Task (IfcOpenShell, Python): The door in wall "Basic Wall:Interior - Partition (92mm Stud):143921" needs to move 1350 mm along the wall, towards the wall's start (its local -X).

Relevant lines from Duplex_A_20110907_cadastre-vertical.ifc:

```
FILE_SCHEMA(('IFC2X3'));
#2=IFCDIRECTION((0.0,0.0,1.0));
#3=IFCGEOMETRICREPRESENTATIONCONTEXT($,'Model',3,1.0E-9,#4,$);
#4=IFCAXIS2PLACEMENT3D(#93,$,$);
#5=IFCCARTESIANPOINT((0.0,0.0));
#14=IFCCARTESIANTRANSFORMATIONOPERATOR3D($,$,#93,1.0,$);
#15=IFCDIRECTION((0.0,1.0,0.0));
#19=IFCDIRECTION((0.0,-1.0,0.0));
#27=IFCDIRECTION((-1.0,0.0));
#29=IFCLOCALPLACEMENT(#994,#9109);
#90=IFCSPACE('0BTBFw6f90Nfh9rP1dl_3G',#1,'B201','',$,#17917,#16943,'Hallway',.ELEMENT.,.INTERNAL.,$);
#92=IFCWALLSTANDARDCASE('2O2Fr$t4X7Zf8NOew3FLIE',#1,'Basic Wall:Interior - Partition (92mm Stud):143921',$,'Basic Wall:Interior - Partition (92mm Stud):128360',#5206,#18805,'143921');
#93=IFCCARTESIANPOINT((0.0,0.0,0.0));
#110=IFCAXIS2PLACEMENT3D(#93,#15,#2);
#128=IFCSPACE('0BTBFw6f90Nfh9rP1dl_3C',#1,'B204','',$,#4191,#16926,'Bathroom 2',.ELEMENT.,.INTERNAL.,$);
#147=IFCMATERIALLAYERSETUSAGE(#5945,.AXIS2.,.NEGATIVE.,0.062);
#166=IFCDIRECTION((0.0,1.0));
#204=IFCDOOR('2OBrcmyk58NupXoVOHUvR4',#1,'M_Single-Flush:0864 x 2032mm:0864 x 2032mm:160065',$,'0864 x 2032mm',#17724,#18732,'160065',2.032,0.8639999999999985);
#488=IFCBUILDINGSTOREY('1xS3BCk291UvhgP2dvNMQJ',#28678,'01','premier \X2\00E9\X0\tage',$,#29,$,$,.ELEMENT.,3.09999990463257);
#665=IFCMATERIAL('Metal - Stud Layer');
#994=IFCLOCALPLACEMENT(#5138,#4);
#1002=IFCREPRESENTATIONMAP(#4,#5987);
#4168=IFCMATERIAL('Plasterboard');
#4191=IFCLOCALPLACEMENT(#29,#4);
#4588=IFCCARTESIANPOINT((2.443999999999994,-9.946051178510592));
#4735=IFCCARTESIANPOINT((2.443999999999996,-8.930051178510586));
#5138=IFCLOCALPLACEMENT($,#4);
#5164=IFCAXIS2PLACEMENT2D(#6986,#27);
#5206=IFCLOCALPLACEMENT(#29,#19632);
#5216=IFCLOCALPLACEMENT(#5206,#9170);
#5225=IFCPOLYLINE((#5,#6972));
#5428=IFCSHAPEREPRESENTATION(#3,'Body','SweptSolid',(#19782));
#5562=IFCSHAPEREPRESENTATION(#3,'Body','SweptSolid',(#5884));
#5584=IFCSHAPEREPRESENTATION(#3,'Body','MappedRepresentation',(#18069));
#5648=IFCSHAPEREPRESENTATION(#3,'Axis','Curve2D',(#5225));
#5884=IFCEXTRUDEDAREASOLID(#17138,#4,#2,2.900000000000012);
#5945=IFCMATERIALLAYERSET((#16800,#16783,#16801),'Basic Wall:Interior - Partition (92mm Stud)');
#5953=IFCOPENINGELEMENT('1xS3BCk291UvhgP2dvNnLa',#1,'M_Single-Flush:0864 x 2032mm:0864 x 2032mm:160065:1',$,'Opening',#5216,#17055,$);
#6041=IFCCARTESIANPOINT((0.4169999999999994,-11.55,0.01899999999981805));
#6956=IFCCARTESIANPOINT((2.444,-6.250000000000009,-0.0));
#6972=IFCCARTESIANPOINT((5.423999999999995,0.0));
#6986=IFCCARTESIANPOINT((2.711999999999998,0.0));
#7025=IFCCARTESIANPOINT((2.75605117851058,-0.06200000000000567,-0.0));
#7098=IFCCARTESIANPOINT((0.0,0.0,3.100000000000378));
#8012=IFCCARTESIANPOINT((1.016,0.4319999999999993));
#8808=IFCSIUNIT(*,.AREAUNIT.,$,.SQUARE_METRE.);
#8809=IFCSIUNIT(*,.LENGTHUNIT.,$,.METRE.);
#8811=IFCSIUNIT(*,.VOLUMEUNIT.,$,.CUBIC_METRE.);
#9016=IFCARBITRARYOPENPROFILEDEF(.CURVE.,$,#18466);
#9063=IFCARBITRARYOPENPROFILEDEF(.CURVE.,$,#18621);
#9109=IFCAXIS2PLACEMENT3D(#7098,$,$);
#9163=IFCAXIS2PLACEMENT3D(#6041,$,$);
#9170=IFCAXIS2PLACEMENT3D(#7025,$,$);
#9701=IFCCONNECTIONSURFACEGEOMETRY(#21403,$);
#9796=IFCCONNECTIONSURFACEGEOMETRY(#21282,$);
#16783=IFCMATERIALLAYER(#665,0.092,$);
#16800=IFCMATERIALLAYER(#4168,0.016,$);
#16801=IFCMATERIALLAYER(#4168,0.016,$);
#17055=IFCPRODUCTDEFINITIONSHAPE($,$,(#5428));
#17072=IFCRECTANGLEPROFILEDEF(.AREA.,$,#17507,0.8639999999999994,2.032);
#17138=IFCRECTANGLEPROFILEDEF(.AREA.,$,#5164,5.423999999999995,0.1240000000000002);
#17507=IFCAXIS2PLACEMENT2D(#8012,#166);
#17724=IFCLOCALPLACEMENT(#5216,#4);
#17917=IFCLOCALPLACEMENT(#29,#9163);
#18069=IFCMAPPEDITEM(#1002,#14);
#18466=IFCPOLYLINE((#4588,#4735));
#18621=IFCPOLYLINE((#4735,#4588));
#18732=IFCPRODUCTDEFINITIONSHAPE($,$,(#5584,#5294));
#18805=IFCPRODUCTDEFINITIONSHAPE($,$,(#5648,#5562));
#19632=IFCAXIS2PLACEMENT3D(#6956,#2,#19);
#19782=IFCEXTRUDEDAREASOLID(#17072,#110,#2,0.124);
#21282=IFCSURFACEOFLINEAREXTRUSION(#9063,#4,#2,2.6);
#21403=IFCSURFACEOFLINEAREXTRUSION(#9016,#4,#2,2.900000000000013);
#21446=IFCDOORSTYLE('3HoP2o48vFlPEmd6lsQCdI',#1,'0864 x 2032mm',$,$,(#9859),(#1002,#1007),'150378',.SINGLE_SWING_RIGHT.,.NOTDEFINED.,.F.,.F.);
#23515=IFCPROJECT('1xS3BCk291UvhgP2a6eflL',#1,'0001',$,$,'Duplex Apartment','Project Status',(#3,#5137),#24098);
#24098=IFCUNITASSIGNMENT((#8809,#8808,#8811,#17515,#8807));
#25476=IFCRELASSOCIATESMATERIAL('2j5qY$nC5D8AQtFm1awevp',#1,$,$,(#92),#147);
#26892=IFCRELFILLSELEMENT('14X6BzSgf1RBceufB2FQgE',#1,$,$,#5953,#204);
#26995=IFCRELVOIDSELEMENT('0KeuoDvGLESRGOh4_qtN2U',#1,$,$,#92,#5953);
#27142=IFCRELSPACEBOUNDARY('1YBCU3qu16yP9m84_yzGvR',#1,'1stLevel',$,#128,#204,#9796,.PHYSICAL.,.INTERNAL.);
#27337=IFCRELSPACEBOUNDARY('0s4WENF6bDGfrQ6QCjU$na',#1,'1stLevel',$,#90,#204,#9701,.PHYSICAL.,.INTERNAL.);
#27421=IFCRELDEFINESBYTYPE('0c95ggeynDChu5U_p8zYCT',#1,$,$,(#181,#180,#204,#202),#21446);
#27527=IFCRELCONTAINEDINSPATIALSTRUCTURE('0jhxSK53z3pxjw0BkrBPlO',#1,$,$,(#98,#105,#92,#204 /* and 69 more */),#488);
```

```python
import numpy as np
import ifcopenshell
import ifcopenshell.api.geometry
import ifcopenshell.util.placement

model = ifcopenshell.open("Duplex_A_20110907_cadastre-vertical.ifc")

door = model.by_guid("2OBrcmyk58NupXoVOHUvR4")
opening = door.FillsVoids[0].RelatingOpeningElement
wall = opening.VoidsElements[0].RelatingBuildingElement

wall_matrix = ifcopenshell.util.placement.get_local_placement(wall.ObjectPlacement)
shift = wall_matrix[:3, 0] * -1.35
before = ifcopenshell.util.placement.get_local_placement(door.ObjectPlacement)[:3, 3].copy()

# The door is placed relative to its opening, so it follows when the opening moves.
matrix = ifcopenshell.util.placement.get_local_placement(opening.ObjectPlacement)
matrix[:3, 3] += shift
ifcopenshell.api.geometry.edit_object_placement(
    model, product=opening, matrix=matrix, is_si=False, should_transform_children=True
)

# Space boundary surfaces are stored in each space's coordinates; move them too.
for rel in door.ProvidesBoundaries:
    if not rel.ConnectionGeometry:
        continue
    surface = rel.ConnectionGeometry.SurfaceOnRelatingElement
    space_matrix = ifcopenshell.util.placement.get_local_placement(rel.RelatingSpace.ObjectPlacement)
    point = np.array(surface.Position.Location.Coordinates) + space_matrix[:3, :3].T @ shift
    surface.Position = model.createIfcAxis2Placement3D(
        model.createIfcCartesianPoint(point.tolist()), surface.Position.Axis, surface.Position.RefDirection
    )

after = ifcopenshell.util.placement.get_local_placement(door.ObjectPlacement)[:3, 3]
print("door moved by", (after - before).round(3) + 0.0)

model.write("Duplex_A_20110907_cadastre-vertical_edited.ifc")
```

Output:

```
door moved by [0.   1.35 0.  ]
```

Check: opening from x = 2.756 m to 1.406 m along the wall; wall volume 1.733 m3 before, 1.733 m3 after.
